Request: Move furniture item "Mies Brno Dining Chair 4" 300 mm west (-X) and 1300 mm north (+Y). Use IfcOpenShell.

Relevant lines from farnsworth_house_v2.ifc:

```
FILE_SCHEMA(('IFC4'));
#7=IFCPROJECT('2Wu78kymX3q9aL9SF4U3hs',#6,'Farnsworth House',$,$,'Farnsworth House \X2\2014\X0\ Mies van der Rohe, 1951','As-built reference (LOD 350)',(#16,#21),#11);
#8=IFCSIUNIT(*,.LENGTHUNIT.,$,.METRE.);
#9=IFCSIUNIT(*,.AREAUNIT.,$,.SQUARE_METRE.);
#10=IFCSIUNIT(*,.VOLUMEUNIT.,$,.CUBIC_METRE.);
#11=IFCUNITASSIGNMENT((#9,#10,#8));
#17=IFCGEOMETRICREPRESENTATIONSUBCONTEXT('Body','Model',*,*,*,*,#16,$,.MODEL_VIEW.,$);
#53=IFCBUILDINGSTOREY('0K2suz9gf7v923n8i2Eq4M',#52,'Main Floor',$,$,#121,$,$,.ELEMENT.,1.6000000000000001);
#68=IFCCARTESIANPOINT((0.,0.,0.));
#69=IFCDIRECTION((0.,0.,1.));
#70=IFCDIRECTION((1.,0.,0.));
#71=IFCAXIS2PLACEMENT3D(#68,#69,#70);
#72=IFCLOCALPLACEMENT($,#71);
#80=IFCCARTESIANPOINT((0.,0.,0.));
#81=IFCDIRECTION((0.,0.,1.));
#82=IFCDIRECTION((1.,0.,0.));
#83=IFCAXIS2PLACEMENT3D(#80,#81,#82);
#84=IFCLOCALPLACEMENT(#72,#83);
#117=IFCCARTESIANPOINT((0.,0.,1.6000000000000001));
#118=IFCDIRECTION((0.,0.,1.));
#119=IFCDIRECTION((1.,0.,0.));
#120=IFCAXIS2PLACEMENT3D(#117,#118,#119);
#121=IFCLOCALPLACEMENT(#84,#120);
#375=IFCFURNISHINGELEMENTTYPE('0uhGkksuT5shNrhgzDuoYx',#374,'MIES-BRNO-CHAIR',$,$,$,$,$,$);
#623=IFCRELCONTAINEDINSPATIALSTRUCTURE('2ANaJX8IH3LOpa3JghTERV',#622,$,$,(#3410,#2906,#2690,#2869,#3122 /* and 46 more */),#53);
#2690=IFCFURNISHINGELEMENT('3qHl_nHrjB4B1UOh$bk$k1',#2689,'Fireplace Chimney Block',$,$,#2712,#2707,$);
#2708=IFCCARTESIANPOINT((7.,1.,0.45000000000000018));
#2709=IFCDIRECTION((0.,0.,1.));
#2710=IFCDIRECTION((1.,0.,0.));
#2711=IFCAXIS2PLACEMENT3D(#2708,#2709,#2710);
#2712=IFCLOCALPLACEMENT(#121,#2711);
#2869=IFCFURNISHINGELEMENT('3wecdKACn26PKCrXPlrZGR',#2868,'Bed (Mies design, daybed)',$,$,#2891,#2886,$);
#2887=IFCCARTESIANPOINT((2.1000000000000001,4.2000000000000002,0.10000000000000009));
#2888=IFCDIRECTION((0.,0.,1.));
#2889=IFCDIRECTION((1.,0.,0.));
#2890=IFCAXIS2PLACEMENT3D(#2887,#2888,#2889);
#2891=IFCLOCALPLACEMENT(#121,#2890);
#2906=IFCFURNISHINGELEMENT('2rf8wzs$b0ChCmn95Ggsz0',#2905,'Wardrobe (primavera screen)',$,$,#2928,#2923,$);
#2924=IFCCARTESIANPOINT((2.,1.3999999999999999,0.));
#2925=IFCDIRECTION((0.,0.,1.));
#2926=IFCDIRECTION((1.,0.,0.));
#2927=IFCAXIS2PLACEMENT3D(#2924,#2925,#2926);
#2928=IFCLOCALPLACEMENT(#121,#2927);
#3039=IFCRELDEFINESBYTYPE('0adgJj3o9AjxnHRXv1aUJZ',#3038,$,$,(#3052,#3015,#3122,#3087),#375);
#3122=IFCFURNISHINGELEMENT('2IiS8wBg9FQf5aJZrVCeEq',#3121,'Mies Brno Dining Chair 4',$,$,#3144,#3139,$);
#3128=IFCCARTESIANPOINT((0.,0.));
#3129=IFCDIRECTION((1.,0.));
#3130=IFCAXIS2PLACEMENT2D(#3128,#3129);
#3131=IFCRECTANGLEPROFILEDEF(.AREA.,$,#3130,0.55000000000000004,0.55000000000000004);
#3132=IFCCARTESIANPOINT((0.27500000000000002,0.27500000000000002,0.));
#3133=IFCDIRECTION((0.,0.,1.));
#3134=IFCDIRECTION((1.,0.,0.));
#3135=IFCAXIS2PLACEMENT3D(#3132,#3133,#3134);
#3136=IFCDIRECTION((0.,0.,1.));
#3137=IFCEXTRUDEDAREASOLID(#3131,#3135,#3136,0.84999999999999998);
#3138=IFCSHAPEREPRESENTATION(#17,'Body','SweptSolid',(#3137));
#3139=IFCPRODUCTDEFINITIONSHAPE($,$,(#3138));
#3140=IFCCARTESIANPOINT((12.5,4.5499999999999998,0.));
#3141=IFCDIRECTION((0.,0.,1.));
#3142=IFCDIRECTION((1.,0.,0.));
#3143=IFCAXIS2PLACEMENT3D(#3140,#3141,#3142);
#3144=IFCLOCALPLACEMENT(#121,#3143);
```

```python
import ifcopenshell
import ifcopenshell.api.geometry
import ifcopenshell.util.placement
import ifcopenshell.util.unit

model = ifcopenshell.open("farnsworth_house_v2.ifc")
unit_scale = ifcopenshell.util.unit.calculate_unit_scale(model)

item = model.by_guid("2IiS8wBg9FQf5aJZrVCeEq")
matrix = ifcopenshell.util.placement.get_local_placement(item.ObjectPlacement)
matrix[0, 3] -= 0.3 / unit_scale
matrix[1, 3] += 1.3 / unit_scale
ifcopenshell.api.geometry.edit_object_placement(model, product=item, matrix=matrix, is_si=False)

print(ifcopenshell.util.placement.get_local_placement(item.ObjectPlacement).round(3) + 0.0)

model.write("farnsworth_house_v2_edited.ifc")
```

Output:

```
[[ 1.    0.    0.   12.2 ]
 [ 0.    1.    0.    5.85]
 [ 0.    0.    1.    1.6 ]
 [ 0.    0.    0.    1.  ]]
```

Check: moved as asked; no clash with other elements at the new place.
